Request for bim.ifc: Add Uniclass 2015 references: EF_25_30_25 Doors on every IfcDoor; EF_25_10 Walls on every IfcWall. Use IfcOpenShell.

First a look at what the model holds.

```python
import ifcopenshell

model = ifcopenshell.open("bim.ifc")
print(model.schema)
print("classifications:", [c.Name for c in model.by_type("IfcClassification")])
for ifc_class in ("IfcDoor", "IfcRoof", "IfcStair", "IfcWall", "IfcWindow"):
    print(ifc_class, len(model.by_type(ifc_class)))
```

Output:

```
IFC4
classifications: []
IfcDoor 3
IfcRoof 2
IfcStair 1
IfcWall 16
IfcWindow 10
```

```python
import ifcopenshell
import ifcopenshell.api.classification

model = ifcopenshell.open("bim.ifc")

system = ifcopenshell.api.classification.add_classification(model, classification="Uniclass 2015")

codes = {
    "IfcDoor": ("EF_25_30_25", "Doors"),
    "IfcWall": ("EF_25_10", "Walls"),
}
for ifc_class, (code, name) in codes.items():
    products = model.by_type(ifc_class)
    ifcopenshell.api.classification.add_reference(
        model, products=products, classification=system, identification=code, name=name
    )
    print(code, len(products))

model.write("bim_v2.ifc")
```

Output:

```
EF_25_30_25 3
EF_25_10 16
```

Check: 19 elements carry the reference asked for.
